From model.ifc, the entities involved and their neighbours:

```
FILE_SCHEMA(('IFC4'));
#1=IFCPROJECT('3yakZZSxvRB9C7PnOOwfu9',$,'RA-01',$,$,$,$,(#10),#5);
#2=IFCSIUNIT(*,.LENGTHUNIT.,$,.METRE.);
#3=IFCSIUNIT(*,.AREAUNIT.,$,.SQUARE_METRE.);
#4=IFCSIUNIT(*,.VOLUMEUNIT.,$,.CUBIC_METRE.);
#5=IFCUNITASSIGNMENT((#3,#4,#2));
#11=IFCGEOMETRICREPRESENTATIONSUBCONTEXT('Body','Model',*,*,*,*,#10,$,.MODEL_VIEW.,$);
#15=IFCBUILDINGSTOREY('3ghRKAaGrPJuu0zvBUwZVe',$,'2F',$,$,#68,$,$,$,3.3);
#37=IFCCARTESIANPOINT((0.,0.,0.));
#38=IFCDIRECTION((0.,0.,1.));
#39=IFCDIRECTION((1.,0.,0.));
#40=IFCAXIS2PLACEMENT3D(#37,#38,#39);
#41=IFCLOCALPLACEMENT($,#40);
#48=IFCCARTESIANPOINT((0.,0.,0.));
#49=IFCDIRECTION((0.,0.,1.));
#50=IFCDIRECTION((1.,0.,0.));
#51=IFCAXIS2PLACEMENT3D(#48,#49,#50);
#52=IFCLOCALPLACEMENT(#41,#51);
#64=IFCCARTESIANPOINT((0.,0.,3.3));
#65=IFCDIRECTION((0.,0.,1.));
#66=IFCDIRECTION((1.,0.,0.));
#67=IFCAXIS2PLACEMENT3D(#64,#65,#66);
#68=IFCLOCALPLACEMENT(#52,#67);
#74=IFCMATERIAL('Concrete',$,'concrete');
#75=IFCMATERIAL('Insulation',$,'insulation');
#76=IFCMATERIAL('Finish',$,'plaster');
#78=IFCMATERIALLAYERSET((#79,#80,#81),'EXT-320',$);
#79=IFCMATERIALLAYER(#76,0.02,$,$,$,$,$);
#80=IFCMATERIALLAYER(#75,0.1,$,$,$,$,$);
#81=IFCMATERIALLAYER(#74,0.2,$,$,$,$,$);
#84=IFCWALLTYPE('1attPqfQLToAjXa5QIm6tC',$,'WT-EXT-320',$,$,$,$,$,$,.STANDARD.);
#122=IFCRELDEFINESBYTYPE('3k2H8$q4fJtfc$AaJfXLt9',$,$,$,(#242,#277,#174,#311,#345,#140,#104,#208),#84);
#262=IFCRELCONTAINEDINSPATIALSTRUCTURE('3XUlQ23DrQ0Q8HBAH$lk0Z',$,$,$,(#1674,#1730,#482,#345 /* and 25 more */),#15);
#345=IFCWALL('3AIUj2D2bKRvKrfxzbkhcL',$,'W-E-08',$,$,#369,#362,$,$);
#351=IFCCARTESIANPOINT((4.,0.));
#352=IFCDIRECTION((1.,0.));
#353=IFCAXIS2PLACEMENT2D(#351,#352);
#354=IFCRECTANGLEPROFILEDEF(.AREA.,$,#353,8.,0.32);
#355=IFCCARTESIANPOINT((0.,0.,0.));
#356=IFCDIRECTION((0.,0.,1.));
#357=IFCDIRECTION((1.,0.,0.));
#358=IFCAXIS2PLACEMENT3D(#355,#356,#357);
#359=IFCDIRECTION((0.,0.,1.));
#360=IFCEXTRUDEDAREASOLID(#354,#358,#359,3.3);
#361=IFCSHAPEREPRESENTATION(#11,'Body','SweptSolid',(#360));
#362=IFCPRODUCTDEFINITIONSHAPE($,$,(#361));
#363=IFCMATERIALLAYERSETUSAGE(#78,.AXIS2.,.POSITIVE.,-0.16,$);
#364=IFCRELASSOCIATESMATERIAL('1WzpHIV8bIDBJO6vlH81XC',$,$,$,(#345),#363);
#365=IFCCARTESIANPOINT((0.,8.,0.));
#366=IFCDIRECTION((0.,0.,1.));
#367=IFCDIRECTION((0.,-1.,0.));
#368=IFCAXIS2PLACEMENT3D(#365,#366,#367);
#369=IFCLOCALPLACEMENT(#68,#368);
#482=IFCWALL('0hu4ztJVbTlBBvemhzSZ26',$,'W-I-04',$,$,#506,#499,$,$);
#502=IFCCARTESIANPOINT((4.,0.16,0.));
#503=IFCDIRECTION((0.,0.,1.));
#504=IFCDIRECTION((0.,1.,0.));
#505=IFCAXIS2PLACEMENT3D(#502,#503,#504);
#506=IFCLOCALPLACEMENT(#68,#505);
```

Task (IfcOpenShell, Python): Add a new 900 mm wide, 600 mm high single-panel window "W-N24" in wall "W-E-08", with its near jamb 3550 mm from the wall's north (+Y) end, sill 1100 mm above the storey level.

```python
import numpy as np
import ifcopenshell
import ifcopenshell.api.feature
import ifcopenshell.api.geometry
import ifcopenshell.api.root
import ifcopenshell.api.spatial
import ifcopenshell.geom
import ifcopenshell.util.element
import ifcopenshell.util.placement
import ifcopenshell.util.representation
import ifcopenshell.util.shape
import ifcopenshell.util.unit

model = ifcopenshell.open("model.ifc")
unit_scale = ifcopenshell.util.unit.calculate_unit_scale(model)
settings = ifcopenshell.geom.settings()


def volume(element):
    """Net volume in cubic metres, openings subtracted."""
    shape = ifcopenshell.geom.create_shape(settings, element)
    return ifcopenshell.util.shape.get_volume(shape.geometry)


wall = model.by_guid("3AIUj2D2bKRvKrfxzbkhcL")
storey = ifcopenshell.util.element.get_container(wall, ifc_class="IfcBuildingStorey")
context = ifcopenshell.util.representation.get_context(model, "Model", "Body", "MODEL_VIEW")
before = volume(wall)

width, height, from_end, sill = 0.9, 0.6, 3.55, 1.1  # metres

# The wall runs along its own X axis, and the end named is its -X end.
wall_shape = ifcopenshell.geom.create_shape(settings, wall)
x, y, z = ifcopenshell.util.shape.get_vertices(wall_shape.geometry).T
start = x.min() + from_end
face, thickness = float(y.min()), float(y.max() - y.min())
wall_matrix = ifcopenshell.util.placement.get_local_placement(wall.ObjectPlacement)
level = ifcopenshell.util.placement.get_local_placement(storey.ObjectPlacement)[2, 3]


def in_wall(x, y):
    """Placement at x, y metres in the wall's axes, at sill height."""
    matrix = wall_matrix.copy()
    matrix[:, 3] = wall_matrix @ np.array([x / unit_scale, y / unit_scale, 0.0, 1.0])
    matrix[2, 3] = level + sill / unit_scale
    return matrix


# Opening: a box that overshoots both wall faces by 50 mm.
opening = ifcopenshell.api.root.create_entity(model, ifc_class="IfcOpeningElement", predefined_type="OPENING")
box = ifcopenshell.api.geometry.add_wall_representation(
    model, context=context, length=width, height=height, thickness=thickness + 0.1
)
ifcopenshell.api.geometry.assign_representation(model, product=opening, representation=box)
ifcopenshell.api.geometry.edit_object_placement(model, product=opening, matrix=in_wall(start, face - 0.05), is_si=False)
ifcopenshell.api.feature.add_feature(model, feature=opening, element=wall)

window = ifcopenshell.api.root.create_entity(model, ifc_class="IfcWindow", name="W-N24", predefined_type="WINDOW")
window.OverallWidth, window.OverallHeight = width / unit_scale, height / unit_scale
window.PartitioningType = "SINGLE_PANEL"
body = ifcopenshell.api.geometry.add_window_representation(
    model,
    context=context,
    overall_width=window.OverallWidth,
    overall_height=window.OverallHeight,
    partition_type="SINGLE_PANEL",
)
ifcopenshell.api.geometry.assign_representation(model, product=window, representation=body)
ifcopenshell.api.spatial.assign_container(model, products=[window], relating_structure=storey)
ifcopenshell.api.feature.add_filling(model, opening=opening, element=window)

# Centre the window in the wall's thickness.
ifcopenshell.api.geometry.edit_object_placement(model, product=window, matrix=in_wall(start, face), is_si=False)
window_shape = ifcopenshell.geom.create_shape(settings, window)
depth = ifcopenshell.util.shape.get_vertices(window_shape.geometry)[:, 1]
offset = face + thickness / 2 - (depth.min() + depth.max()) / 2
ifcopenshell.api.geometry.edit_object_placement(model, product=window, matrix=in_wall(start, offset), is_si=False)

after = volume(wall)

print(f"wall volume {before:.3f} -> {after:.3f} m3")

model.write("model_v2.ifc")
```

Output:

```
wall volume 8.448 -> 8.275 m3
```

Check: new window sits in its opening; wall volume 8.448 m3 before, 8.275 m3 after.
